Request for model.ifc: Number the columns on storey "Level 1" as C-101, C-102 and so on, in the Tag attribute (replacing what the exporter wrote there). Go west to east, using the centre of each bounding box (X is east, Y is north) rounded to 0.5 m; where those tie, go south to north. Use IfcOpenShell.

First a look at what the model holds.

```python
import ifcopenshell
import ifcopenshell.util.element
import ifcopenshell.util.placement

model = ifcopenshell.open("model.ifc")
print(model.schema)
storey = next(s for s in model.by_type("IfcBuildingStorey") if s.Name == "Level 1")
columns = [e for e in ifcopenshell.util.element.get_decomposition(storey) if e.is_a("IfcColumn")]
for e in sorted(columns, key=lambda e: e.id()):
    origin = ifcopenshell.util.placement.get_local_placement(e.ObjectPlacement)[:3, 3]
    print(e.id(), e.Tag, e.Name, origin.round(2) + 0.0, sep=" | ")
```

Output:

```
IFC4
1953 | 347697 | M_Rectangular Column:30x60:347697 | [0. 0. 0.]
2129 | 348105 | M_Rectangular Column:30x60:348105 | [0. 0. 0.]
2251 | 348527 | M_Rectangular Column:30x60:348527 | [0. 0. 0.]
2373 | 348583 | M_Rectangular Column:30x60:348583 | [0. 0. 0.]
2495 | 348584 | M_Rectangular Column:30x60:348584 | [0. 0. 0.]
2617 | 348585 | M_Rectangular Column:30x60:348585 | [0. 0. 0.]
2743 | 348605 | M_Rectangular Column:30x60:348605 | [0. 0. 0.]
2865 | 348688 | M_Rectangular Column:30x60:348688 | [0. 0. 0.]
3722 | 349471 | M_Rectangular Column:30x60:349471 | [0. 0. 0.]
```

```python
import ifcopenshell
import ifcopenshell.geom
import ifcopenshell.util.element
import ifcopenshell.util.shape

model = ifcopenshell.open("model.ifc")
settings = ifcopenshell.geom.settings()
settings.set("use-world-coords", True)


def centre(element):
    shape = ifcopenshell.geom.create_shape(settings, element)
    return ifcopenshell.util.shape.get_bbox_centroid(shape.geometry)


storey = next(s for s in model.by_type("IfcBuildingStorey") if s.Name == "Level 1")
columns = [e for e in ifcopenshell.util.element.get_decomposition(storey) if e.is_a("IfcColumn")]

# Insertion points can sit at a corner or the storey origin, so sort by the geometry (in metres).
centres = {e: centre(e) for e in columns}
columns.sort(key=lambda e: (round(centres[e][0] / 0.5), centres[e][1]))

for i, e in enumerate(columns, start=1):
    number = f"C-1{i:02d}"
    e.Tag = number
    print(e.id(), number)

model.write("model-out.ifc")
```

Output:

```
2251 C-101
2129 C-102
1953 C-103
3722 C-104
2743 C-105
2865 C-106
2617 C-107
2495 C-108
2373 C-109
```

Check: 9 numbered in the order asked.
